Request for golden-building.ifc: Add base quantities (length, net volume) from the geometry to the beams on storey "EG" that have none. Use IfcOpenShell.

First a look at what the model holds.

```python
import ifcopenshell
import ifcopenshell.util.element
import ifcopenshell.util.unit

model = ifcopenshell.open("golden-building.ifc")
print(model.schema)
for unit_type in ("LENGTHUNIT", "AREAUNIT", "VOLUMEUNIT"):
    print(unit_type, ifcopenshell.util.unit.calculate_unit_scale(model, unit_type))
storey = next(s for s in model.by_type("IfcBuildingStorey") if s.Name == "EG")
beams = [e for e in ifcopenshell.util.element.get_decomposition(storey) if e.is_a("IfcBeam")]
for e in sorted(beams, key=lambda e: e.id()):
    print(e.id(), e.is_a(), e.Name, list(ifcopenshell.util.element.get_psets(e, qtos_only=True)), sep=" | ")
```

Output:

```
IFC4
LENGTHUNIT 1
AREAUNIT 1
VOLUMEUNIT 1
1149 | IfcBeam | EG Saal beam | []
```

```python
import ifcopenshell
import ifcopenshell.api.pset
import ifcopenshell.geom
import ifcopenshell.util.element
import ifcopenshell.util.shape
import ifcopenshell.util.unit

model = ifcopenshell.open("golden-building.ifc")
unit_scale = ifcopenshell.util.unit.calculate_unit_scale(model)
volume_scale = ifcopenshell.util.unit.calculate_unit_scale(model, "VOLUMEUNIT")
settings = ifcopenshell.geom.settings()

storey = next(s for s in model.by_type("IfcBuildingStorey") if s.Name == "EG")
beams = [e for e in ifcopenshell.util.element.get_decomposition(storey) if e.is_a("IfcBeam")]

for e in sorted(beams, key=lambda e: e.id()):
    if ifcopenshell.util.element.get_psets(e, qtos_only=True, should_inherit=False):
        continue
    # Geometry comes back in metres, in the element's own axes.
    shape = ifcopenshell.geom.create_shape(settings, e)
    values = {
        "Length": ifcopenshell.util.shape.get_max_xyz(shape.geometry) / unit_scale,
        "NetVolume": ifcopenshell.util.shape.get_volume(shape.geometry) / volume_scale,
    }
    qto = ifcopenshell.api.pset.add_qto(model, product=e, name="Qto_BeamBaseQuantities")
    ifcopenshell.api.pset.edit_qto(model, qto=qto, properties=values)
    print(e.id(), {k: round(v, 3) for k, v in values.items()})

model.write("golden-building-out.ifc")
```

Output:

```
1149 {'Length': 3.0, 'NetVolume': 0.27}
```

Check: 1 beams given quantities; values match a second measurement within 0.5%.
